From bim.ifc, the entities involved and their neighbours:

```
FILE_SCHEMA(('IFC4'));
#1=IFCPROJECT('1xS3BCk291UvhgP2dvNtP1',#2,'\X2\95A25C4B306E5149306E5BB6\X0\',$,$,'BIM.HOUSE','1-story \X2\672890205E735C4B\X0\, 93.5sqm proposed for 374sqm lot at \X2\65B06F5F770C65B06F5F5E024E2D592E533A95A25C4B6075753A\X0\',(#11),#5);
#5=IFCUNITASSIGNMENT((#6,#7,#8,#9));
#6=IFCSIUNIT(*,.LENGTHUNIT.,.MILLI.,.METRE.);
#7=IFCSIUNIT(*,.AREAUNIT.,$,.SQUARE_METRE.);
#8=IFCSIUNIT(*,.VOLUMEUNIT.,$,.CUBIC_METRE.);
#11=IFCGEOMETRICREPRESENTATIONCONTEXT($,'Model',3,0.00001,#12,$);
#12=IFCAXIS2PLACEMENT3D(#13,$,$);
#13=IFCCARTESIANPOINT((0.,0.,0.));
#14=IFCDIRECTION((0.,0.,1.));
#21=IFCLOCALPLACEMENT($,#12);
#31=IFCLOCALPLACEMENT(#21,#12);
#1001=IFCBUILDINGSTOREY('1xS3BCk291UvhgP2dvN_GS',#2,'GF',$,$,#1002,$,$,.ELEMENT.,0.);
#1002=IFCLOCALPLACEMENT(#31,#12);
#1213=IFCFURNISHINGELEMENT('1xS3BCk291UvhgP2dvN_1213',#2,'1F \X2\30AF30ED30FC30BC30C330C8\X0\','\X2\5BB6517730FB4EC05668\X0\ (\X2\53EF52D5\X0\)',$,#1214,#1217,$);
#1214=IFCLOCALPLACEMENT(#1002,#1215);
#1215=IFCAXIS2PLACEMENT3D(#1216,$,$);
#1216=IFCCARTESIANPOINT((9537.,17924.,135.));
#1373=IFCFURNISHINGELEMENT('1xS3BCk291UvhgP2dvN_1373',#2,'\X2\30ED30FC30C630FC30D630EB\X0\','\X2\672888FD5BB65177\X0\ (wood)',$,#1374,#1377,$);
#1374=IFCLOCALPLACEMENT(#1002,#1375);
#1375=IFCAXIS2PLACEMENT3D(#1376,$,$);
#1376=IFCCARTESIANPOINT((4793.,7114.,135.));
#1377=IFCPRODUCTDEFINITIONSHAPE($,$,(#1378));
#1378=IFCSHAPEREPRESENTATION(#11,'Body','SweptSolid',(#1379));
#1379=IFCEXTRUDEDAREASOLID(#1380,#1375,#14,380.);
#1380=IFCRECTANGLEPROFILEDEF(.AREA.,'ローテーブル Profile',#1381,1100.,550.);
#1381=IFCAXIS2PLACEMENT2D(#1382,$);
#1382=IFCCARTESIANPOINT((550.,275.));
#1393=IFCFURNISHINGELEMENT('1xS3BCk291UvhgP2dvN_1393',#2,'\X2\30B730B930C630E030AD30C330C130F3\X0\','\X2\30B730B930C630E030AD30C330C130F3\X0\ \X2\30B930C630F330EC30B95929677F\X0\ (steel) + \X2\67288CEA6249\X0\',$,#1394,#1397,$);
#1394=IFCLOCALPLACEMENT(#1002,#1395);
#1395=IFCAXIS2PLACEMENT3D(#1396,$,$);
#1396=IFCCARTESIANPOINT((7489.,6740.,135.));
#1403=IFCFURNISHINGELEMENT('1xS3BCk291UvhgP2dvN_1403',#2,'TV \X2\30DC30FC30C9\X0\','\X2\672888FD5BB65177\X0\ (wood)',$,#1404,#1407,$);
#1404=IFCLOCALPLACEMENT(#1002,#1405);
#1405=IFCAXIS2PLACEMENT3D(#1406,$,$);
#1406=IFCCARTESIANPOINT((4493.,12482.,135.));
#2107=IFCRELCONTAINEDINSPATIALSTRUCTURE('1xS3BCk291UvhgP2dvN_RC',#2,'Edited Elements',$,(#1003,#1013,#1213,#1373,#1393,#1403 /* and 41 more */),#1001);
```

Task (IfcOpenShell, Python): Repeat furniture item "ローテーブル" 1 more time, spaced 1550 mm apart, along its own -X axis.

```python
import ifcopenshell
import ifcopenshell.api.geometry
import ifcopenshell.api.root
import ifcopenshell.util.element
import ifcopenshell.util.placement

model = ifcopenshell.open("bim.ifc")


def reuse_history(source, copy):
    """copy_class also copies each property set's owner history, people and application; keep the originals."""
    for rel in copy.IsDefinedBy:
        if rel.is_a("IfcRelDefinesByProperties") and (history := rel.RelatingPropertyDefinition.OwnerHistory):
            rel.RelatingPropertyDefinition.OwnerHistory = source.OwnerHistory
            ifcopenshell.util.element.remove_deep2(model, history)


source = model.by_id(1373)
base = ifcopenshell.util.placement.get_local_placement(source.ObjectPlacement)
step = -base[:3, 0] * 1550.0

for i in range(1, 2):
    copy = ifcopenshell.api.root.copy_class(model, product=source)
    copy.Representation = ifcopenshell.util.element.copy_deep(
        model, source.Representation, exclude=["IfcGeometricRepresentationContext", "IfcRepresentationMap"]
    )
    reuse_history(source, copy)
    matrix = base.copy()
    matrix[:3, 3] += i * step
    print("added at", matrix[:3, 3].round(3) + 0.0)
    ifcopenshell.api.geometry.edit_object_placement(model, product=copy, matrix=matrix, is_si=False)

model.write("bim-out.ifc")
```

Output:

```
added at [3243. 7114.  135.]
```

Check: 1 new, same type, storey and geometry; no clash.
